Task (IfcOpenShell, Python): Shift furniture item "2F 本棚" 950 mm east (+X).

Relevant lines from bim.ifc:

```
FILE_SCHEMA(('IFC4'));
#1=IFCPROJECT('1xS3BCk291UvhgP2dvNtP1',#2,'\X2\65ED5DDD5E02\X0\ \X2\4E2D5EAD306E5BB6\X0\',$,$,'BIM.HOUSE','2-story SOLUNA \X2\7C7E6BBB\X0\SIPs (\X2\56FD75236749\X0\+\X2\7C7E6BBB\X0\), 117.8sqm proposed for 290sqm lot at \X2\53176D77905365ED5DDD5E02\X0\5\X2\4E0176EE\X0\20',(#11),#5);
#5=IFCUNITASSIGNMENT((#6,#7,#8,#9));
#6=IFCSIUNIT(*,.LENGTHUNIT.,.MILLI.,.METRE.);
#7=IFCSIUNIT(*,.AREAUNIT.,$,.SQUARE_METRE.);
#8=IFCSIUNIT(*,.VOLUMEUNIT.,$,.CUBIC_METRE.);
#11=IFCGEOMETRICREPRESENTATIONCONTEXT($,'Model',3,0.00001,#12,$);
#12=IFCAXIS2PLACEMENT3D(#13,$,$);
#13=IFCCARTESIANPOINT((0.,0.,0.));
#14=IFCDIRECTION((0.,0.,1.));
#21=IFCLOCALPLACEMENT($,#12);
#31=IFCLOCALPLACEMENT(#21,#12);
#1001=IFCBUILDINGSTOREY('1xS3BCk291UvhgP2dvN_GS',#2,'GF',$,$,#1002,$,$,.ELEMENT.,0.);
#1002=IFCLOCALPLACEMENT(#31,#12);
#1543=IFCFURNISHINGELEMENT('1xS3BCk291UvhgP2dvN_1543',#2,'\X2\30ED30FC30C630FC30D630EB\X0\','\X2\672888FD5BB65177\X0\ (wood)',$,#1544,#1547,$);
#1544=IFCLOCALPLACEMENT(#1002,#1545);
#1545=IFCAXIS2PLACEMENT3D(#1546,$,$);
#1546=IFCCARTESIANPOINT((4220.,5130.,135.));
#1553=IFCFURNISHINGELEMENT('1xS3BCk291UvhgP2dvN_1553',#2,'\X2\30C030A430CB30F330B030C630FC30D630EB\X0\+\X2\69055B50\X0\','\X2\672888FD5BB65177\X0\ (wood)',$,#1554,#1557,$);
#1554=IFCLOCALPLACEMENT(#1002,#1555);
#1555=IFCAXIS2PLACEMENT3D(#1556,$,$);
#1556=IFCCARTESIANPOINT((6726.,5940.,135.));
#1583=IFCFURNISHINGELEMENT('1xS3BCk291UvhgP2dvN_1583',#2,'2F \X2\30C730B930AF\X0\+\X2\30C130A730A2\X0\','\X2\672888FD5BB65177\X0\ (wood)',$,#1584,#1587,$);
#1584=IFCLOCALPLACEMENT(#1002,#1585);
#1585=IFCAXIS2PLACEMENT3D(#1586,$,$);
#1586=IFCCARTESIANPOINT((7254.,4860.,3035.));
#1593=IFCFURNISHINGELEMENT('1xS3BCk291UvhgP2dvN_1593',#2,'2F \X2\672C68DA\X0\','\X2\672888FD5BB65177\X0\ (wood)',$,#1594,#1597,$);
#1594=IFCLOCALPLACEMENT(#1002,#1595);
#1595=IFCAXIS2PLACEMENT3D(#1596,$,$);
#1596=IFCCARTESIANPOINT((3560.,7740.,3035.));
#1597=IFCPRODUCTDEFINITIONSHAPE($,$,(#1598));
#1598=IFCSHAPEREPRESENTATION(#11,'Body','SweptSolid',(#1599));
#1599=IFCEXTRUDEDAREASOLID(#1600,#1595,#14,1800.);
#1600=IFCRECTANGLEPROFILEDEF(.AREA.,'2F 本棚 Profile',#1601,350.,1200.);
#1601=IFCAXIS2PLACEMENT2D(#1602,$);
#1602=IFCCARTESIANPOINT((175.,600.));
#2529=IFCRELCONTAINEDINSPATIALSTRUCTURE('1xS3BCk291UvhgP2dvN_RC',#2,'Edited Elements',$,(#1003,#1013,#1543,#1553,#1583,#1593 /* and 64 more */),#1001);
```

```python
import ifcopenshell
import ifcopenshell.api.geometry
import ifcopenshell.util.placement
import ifcopenshell.util.unit

model = ifcopenshell.open("bim.ifc")
unit_scale = ifcopenshell.util.unit.calculate_unit_scale(model)

item = model.by_guid("1xS3BCk291UvhgP2dvN_1593")
matrix = ifcopenshell.util.placement.get_local_placement(item.ObjectPlacement)
matrix[0, 3] += 0.95 / unit_scale
ifcopenshell.api.geometry.edit_object_placement(model, product=item, matrix=matrix, is_si=False)

print(ifcopenshell.util.placement.get_local_placement(item.ObjectPlacement).round(3) + 0.0)

model.write("bim-out.ifc")
```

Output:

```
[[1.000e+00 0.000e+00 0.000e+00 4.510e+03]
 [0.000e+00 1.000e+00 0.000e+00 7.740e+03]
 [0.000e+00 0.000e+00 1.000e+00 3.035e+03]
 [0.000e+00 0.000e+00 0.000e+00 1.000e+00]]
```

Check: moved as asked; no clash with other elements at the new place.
